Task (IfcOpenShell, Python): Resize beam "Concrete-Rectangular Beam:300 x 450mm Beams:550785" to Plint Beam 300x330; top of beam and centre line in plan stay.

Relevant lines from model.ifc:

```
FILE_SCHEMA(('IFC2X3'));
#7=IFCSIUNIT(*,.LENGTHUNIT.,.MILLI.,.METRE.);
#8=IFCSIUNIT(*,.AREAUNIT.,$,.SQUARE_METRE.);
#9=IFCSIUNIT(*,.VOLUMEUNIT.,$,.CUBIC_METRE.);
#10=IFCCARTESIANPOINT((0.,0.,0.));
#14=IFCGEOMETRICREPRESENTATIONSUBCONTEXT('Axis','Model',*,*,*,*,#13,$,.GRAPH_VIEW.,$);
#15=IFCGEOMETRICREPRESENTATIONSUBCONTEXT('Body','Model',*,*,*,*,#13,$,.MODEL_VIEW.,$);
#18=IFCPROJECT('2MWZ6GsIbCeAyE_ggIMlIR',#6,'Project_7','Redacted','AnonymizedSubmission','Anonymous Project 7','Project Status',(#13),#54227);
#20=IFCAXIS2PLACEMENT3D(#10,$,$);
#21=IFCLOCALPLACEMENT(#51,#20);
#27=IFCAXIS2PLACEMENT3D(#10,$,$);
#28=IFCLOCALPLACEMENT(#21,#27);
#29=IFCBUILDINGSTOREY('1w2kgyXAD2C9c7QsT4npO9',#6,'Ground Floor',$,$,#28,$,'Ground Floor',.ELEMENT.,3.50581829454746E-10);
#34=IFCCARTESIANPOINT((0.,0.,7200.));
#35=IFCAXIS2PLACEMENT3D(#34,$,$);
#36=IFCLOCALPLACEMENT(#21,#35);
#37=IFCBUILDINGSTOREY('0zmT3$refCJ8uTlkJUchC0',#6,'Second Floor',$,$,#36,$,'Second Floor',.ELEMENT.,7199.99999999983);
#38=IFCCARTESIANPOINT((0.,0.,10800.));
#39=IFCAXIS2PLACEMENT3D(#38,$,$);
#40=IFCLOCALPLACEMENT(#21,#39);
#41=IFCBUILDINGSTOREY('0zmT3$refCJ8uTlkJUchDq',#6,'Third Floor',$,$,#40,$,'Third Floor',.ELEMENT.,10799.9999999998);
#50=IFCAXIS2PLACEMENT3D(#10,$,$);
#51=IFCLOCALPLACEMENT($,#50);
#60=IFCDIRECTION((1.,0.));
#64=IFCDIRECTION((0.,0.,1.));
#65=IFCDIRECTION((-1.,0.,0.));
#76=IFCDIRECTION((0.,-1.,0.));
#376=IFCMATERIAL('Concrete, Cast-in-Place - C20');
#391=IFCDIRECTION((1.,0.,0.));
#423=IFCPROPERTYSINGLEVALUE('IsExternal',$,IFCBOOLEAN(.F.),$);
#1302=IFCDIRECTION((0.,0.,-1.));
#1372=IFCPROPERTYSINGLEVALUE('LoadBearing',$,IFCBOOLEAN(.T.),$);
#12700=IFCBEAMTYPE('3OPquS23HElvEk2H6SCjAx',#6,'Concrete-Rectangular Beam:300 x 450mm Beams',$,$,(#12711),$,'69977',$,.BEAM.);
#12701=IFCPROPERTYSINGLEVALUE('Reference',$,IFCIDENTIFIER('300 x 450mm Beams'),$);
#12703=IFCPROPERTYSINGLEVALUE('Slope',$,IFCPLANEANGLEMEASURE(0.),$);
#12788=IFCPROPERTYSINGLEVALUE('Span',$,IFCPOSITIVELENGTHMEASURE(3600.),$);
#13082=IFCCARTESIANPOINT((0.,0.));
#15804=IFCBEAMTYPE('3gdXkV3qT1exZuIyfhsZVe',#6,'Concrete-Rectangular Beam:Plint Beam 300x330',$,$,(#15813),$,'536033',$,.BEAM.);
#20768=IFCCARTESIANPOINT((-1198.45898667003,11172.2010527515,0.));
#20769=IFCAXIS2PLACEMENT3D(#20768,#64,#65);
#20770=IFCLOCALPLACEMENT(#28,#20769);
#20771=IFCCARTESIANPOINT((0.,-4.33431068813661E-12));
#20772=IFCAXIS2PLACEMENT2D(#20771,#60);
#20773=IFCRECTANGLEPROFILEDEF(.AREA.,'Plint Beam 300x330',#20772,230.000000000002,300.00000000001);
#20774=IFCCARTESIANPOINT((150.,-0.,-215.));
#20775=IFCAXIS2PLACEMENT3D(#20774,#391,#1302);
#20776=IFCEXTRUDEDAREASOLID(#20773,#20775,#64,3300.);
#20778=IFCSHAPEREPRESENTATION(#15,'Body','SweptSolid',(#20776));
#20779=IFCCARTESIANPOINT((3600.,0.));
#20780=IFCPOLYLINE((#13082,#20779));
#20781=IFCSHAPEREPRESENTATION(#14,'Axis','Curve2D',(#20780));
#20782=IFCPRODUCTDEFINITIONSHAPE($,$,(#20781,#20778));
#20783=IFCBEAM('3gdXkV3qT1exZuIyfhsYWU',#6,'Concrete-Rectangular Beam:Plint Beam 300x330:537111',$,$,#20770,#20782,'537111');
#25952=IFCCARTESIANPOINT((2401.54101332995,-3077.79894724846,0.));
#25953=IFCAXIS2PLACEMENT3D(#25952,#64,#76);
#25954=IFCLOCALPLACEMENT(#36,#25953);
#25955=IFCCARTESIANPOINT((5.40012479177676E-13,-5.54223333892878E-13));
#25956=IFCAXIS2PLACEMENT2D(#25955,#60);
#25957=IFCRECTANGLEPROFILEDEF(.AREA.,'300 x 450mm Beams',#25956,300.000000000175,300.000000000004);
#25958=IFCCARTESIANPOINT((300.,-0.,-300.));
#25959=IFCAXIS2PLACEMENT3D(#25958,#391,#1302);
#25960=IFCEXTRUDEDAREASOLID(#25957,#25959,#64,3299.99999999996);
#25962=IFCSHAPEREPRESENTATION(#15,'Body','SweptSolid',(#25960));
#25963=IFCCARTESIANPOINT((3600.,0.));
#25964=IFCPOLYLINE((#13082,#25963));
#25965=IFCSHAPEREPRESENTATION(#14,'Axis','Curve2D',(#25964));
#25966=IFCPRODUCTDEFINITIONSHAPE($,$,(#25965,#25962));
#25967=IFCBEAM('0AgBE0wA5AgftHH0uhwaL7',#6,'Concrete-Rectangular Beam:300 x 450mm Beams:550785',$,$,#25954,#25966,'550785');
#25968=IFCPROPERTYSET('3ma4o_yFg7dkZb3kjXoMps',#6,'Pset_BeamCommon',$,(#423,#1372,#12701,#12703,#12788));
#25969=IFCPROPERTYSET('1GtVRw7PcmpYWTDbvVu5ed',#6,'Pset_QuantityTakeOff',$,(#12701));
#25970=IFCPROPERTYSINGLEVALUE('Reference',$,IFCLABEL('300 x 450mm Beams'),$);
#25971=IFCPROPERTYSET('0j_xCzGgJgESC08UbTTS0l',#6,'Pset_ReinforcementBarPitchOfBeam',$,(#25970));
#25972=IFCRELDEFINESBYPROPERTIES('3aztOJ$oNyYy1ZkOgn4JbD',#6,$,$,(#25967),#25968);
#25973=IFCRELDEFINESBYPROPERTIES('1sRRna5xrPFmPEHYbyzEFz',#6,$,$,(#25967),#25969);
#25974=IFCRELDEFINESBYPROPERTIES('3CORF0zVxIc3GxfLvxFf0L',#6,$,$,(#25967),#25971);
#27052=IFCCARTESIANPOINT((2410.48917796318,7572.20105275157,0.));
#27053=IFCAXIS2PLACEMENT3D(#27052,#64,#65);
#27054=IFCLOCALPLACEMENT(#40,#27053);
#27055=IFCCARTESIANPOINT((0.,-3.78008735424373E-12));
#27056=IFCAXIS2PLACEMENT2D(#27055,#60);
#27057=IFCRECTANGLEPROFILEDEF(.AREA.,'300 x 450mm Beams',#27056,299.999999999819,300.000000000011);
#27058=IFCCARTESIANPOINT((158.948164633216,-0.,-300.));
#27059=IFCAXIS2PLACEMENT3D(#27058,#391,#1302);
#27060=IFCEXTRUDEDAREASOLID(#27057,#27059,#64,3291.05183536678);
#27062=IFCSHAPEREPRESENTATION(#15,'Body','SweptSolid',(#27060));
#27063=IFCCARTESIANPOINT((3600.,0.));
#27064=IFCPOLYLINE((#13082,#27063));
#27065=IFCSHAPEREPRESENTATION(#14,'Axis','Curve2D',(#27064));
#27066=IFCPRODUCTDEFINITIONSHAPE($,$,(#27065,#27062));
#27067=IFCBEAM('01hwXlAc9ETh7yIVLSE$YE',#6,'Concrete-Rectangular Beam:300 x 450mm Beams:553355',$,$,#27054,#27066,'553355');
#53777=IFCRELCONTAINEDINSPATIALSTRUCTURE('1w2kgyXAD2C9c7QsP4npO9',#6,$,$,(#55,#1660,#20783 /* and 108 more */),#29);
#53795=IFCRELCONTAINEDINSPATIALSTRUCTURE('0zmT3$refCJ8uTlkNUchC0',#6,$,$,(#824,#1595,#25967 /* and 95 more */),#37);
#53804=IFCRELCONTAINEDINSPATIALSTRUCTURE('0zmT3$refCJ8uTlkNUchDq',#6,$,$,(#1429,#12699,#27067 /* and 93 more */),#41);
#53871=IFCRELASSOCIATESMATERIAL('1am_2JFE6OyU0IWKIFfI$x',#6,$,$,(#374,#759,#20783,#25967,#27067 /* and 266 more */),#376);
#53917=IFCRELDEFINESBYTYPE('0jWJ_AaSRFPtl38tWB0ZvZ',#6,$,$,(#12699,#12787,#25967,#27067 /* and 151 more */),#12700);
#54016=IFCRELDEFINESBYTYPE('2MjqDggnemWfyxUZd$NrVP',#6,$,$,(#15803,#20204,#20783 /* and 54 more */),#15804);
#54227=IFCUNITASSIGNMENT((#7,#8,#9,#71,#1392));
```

```python
import ifcopenshell
import ifcopenshell.api.pset
import ifcopenshell.api.type
import ifcopenshell.util.element
import ifcopenshell.util.representation

model = ifcopenshell.open("model.ifc")

member = model.by_id(25967)
source = next(p for p in model.by_type("IfcRectangleProfileDef") if p.ProfileName == "Plint Beam 300x330")

body = ifcopenshell.util.representation.get_representation(member, "Model", "Body")
solid = body.Items[0]
old_profile = solid.SweptArea

# Copy the section's sizes but keep this member's own profile position.
profile = ifcopenshell.util.element.copy(model, source)
# Profiles are centred, so shift by half the change in depth to hold the top.
shift = (old_profile.XDim - profile.XDim) / 2
x, y = old_profile.Position.Location.Coordinates
up = (-1.0, 0.0)  # upwards, in the solid's own plane
location = model.createIfcCartesianPoint((x + up[0] * shift, y + up[1] * shift))
profile.Position = model.createIfcAxis2Placement2D(location, old_profile.Position.RefDirection)
solid.SweptArea = profile
if not model.get_total_inverses(old_profile):
    ifcopenshell.util.element.remove_deep2(model, old_profile)

new_type = model.by_guid("3gdXkV3qT1exZuIyfhsZVe")
ifcopenshell.api.type.assign_type(
    model, related_objects=[member], relating_type=new_type, should_map_representations=False
)
member.Name = member.Name.replace("300 x 450mm Beams", "Plint Beam 300x330")
pset = model.by_id(ifcopenshell.util.element.get_pset(member, "Pset_BeamCommon", should_inherit=False)["id"])
ifcopenshell.api.pset.edit_pset(model, pset=pset, properties={"Reference": "Plint Beam 300x330"})
pset = model.by_id(ifcopenshell.util.element.get_pset(member, "Pset_QuantityTakeOff", should_inherit=False)["id"])
ifcopenshell.api.pset.edit_pset(model, pset=pset, properties={"Reference": "Plint Beam 300x330"})
pset = model.by_id(ifcopenshell.util.element.get_pset(member, "Pset_ReinforcementBarPitchOfBeam", should_inherit=False)["id"])
ifcopenshell.api.pset.edit_pset(model, pset=pset, properties={"Reference": "Plint Beam 300x330"})

print(solid.SweptArea)

model.write("model_v2.ifc")
```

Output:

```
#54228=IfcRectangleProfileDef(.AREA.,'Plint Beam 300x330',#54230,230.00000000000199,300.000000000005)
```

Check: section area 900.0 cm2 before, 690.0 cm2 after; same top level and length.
